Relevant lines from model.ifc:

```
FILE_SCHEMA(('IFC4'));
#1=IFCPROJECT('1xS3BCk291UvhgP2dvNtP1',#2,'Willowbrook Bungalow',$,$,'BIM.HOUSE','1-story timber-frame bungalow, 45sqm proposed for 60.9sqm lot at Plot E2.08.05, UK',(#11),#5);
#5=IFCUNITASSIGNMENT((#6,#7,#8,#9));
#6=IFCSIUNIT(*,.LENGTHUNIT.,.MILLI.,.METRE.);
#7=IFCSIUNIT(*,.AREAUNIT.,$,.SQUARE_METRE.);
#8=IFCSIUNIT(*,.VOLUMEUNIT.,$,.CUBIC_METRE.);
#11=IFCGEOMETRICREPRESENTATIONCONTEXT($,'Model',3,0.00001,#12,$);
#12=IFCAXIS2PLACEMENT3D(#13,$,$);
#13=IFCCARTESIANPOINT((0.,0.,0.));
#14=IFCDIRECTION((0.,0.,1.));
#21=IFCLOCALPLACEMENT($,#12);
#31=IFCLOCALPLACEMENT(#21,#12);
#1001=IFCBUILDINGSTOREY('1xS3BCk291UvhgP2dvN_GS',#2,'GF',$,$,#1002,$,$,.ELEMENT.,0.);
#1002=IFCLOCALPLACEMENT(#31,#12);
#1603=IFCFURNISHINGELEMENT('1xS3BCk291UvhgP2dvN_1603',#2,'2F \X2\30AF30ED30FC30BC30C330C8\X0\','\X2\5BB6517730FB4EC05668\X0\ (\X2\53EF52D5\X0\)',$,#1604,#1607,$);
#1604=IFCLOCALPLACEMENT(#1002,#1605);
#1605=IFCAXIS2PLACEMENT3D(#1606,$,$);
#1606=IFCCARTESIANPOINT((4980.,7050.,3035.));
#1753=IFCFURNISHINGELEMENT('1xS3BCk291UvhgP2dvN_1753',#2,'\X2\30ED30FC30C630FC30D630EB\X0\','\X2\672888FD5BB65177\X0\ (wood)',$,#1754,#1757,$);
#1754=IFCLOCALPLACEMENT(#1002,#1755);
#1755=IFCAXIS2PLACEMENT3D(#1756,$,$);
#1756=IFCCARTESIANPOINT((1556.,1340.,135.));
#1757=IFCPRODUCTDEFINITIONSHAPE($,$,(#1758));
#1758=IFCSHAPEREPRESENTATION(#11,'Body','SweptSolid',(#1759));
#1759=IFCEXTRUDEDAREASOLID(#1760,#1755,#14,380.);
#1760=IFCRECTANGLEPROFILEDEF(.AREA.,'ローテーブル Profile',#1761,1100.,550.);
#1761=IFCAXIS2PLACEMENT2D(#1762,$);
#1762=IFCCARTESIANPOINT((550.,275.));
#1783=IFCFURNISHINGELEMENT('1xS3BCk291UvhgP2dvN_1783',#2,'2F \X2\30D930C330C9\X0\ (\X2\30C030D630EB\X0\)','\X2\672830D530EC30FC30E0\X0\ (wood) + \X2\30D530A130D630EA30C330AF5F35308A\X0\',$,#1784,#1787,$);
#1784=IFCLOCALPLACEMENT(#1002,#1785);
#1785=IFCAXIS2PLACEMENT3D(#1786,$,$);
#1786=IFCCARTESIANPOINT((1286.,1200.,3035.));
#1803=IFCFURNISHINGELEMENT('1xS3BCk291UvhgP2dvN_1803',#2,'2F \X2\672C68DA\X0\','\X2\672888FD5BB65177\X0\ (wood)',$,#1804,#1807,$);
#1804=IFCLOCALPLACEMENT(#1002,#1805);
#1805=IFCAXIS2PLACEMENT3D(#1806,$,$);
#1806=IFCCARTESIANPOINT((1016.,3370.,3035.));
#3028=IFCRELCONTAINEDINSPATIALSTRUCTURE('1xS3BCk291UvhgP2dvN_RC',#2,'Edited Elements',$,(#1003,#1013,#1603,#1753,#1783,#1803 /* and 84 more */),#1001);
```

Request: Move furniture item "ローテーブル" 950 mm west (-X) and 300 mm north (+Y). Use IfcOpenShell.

```python
import ifcopenshell
import ifcopenshell.api.geometry
import ifcopenshell.util.placement

model = ifcopenshell.open("model.ifc")

item = model.by_guid("1xS3BCk291UvhgP2dvN_1753")
matrix = ifcopenshell.util.placement.get_local_placement(item.ObjectPlacement)
matrix[0, 3] -= 950.0
matrix[1, 3] += 300.0
ifcopenshell.api.geometry.edit_object_placement(model, product=item, matrix=matrix, is_si=False)

print(ifcopenshell.util.placement.get_local_placement(item.ObjectPlacement).round(3) + 0.0)

model.write("model_rev.ifc")
```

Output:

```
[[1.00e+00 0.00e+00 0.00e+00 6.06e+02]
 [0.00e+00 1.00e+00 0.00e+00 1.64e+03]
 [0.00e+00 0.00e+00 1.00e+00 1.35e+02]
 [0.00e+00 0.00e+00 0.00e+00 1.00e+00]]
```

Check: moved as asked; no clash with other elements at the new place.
